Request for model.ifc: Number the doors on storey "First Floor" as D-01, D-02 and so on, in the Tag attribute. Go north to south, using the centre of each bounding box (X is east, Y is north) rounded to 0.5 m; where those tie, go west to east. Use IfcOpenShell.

First a look at what the model holds.

```python
import ifcopenshell
import ifcopenshell.util.element
import ifcopenshell.util.placement

model = ifcopenshell.open("model.ifc")
print(model.schema)
storey = next(s for s in model.by_type("IfcBuildingStorey") if s.Name == "First Floor")
doors = [e for e in ifcopenshell.util.element.get_decomposition(storey) if e.is_a("IfcDoor")]
for e in sorted(doors, key=lambda e: e.id()):
    origin = ifcopenshell.util.placement.get_local_placement(e.ObjectPlacement)[:3, 3]
    print(e.id(), e.Tag, e.Name, origin.round(2) + 0.0, sep=" | ")
```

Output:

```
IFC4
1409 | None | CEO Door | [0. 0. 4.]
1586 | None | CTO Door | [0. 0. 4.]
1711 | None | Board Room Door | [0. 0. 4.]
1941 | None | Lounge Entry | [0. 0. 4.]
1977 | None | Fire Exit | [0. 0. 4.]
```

```python
import ifcopenshell
import ifcopenshell.geom
import ifcopenshell.util.element
import ifcopenshell.util.shape

model = ifcopenshell.open("model.ifc")
settings = ifcopenshell.geom.settings()
settings.set("use-world-coords", True)


def centre(element):
    shape = ifcopenshell.geom.create_shape(settings, element)
    return ifcopenshell.util.shape.get_bbox_centroid(shape.geometry)


storey = next(s for s in model.by_type("IfcBuildingStorey") if s.Name == "First Floor")
doors = [e for e in ifcopenshell.util.element.get_decomposition(storey) if e.is_a("IfcDoor")]

# Insertion points can sit at a corner or the storey origin, so sort by the geometry (in metres).
centres = {e: centre(e) for e in doors}
doors.sort(key=lambda e: (-round(centres[e][1] / 0.5), centres[e][0]))

for i, e in enumerate(doors, start=1):
    number = f"D-{i:02d}"
    e.Tag = number
    print(e.id(), number)

model.write("model_rev.ifc")
```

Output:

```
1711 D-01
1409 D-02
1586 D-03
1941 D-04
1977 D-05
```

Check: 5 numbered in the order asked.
